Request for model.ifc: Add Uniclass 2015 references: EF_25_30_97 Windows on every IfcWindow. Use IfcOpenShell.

First a look at what the model holds.

```python
import ifcopenshell

model = ifcopenshell.open("model.ifc")
print(model.schema)
print("classifications:", [c.Name for c in model.by_type("IfcClassification")])
for ifc_class in ("IfcDoor", "IfcRoof", "IfcStair", "IfcWall", "IfcWindow"):
    print(ifc_class, len(model.by_type(ifc_class)))
```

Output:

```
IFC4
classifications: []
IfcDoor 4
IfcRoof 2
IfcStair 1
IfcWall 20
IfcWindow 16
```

```python
import ifcopenshell
import ifcopenshell.api.classification

model = ifcopenshell.open("model.ifc")

system = ifcopenshell.api.classification.add_classification(model, classification="Uniclass 2015")

codes = {
    "IfcWindow": ("EF_25_30_97", "Windows"),
}
for ifc_class, (code, name) in codes.items():
    products = model.by_type(ifc_class)
    ifcopenshell.api.classification.add_reference(
        model, products=products, classification=system, identification=code, name=name
    )
    print(code, len(products))

model.write("model_rev.ifc")
```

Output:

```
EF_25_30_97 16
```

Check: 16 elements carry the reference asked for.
